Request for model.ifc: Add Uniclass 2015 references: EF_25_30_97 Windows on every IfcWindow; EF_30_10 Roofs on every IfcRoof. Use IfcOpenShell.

First a look at what the model holds.

```python
import ifcopenshell

model = ifcopenshell.open("model.ifc")
print(model.schema)
print("classifications:", [c.Name for c in model.by_type("IfcClassification")])
for ifc_class in ("IfcDoor", "IfcRoof", "IfcStair", "IfcWall", "IfcWindow"):
    print(ifc_class, len(model.by_type(ifc_class)))
```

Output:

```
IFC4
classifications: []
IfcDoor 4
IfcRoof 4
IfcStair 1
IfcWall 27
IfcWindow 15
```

```python
import ifcopenshell
import ifcopenshell.api.classification

model = ifcopenshell.open("model.ifc")

system = ifcopenshell.api.classification.add_classification(model, classification="Uniclass 2015")

codes = {
    "IfcWindow": ("EF_25_30_97", "Windows"),
    "IfcRoof": ("EF_30_10", "Roofs"),
}
for ifc_class, (code, name) in codes.items():
    products = model.by_type(ifc_class)
    ifcopenshell.api.classification.add_reference(
        model, products=products, classification=system, identification=code, name=name
    )
    print(code, len(products))

model.write("model_updated.ifc")
```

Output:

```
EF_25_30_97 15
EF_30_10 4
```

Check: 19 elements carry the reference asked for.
